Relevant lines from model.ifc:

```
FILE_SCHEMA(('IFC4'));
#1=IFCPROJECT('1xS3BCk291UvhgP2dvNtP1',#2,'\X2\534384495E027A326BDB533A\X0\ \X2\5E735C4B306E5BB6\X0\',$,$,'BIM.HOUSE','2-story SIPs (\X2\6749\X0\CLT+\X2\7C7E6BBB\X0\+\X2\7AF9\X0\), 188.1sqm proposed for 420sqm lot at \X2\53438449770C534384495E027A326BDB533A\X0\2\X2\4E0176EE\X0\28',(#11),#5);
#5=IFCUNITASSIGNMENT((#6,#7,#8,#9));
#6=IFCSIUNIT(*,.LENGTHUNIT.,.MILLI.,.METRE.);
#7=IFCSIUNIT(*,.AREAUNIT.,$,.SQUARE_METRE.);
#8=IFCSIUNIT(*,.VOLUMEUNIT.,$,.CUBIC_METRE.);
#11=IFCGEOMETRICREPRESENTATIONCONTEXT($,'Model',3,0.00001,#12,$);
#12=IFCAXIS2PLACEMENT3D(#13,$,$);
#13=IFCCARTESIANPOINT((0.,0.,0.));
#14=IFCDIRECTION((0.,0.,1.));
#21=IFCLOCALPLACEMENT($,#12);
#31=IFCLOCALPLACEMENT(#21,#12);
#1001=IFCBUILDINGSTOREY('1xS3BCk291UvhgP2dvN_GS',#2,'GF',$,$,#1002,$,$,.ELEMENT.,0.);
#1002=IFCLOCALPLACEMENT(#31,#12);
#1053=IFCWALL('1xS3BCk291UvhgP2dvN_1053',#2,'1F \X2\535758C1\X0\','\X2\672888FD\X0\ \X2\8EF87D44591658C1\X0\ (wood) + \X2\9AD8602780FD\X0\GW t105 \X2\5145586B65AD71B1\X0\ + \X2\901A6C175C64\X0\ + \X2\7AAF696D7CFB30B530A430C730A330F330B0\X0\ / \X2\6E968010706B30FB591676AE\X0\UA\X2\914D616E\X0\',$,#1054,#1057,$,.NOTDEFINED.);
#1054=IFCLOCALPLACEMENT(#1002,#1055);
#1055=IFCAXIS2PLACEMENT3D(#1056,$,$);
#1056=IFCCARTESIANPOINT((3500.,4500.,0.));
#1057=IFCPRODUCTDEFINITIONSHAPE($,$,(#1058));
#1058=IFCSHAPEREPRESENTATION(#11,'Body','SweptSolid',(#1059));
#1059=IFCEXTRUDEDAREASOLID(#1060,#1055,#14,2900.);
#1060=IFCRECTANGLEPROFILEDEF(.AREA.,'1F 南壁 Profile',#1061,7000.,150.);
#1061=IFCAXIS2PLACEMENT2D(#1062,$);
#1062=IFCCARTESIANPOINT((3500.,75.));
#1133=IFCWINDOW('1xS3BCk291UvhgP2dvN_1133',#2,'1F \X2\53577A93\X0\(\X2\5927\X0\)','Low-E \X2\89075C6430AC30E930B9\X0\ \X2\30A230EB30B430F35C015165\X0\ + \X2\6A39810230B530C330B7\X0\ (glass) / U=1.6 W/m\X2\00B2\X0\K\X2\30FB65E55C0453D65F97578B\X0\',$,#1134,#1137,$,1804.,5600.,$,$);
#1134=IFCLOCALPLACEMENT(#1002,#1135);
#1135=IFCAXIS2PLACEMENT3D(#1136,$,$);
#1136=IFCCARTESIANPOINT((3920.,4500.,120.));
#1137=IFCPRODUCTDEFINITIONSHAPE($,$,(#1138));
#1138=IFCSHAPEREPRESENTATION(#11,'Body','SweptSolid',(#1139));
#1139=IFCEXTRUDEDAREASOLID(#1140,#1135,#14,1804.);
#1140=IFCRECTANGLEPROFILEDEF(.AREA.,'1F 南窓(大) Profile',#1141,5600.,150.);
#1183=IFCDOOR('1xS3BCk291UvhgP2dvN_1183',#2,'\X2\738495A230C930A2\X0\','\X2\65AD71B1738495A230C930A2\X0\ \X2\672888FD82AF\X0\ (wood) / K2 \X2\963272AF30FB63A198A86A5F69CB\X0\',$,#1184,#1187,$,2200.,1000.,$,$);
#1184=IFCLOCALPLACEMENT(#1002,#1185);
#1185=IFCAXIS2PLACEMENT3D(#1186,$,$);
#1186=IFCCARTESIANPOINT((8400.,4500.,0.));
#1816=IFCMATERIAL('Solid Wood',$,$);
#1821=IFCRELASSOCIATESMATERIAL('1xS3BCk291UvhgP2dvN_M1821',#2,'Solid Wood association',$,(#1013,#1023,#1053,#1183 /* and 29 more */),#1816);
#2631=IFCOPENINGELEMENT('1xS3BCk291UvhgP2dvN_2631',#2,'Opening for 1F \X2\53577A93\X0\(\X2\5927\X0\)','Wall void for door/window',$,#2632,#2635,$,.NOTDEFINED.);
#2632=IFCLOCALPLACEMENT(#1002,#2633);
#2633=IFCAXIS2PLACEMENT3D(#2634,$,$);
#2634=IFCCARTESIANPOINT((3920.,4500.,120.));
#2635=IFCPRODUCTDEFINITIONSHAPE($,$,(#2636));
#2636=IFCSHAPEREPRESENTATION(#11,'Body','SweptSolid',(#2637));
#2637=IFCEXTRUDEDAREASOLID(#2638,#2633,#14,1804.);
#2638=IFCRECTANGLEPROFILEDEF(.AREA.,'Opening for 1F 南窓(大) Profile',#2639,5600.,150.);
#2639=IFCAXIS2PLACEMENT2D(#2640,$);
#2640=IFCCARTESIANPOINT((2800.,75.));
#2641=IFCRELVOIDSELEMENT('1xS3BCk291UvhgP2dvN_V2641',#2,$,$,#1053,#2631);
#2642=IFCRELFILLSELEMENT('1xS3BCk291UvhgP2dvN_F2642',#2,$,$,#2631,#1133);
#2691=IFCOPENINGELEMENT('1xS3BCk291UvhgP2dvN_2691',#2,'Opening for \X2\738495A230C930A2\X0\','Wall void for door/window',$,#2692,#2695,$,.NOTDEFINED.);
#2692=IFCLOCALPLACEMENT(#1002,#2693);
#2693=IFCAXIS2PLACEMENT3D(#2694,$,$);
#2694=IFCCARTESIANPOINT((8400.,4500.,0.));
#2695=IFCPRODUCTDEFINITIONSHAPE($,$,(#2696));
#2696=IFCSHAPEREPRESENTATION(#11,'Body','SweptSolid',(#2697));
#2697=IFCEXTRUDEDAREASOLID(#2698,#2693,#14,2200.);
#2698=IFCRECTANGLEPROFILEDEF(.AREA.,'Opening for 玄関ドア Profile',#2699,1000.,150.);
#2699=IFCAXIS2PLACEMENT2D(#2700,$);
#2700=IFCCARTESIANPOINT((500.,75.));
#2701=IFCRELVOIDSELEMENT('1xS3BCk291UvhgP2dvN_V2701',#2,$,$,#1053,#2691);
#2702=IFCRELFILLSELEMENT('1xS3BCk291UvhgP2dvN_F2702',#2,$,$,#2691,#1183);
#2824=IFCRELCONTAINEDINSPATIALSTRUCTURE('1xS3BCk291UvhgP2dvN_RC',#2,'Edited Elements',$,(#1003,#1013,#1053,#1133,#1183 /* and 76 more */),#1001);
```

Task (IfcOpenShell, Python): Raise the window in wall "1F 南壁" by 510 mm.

```python
import numpy as np
import ifcopenshell
import ifcopenshell.api.geometry
import ifcopenshell.util.placement
import ifcopenshell.util.unit

model = ifcopenshell.open("model.ifc")
unit_scale = ifcopenshell.util.unit.calculate_unit_scale(model)

window = model.by_guid("1xS3BCk291UvhgP2dvN_1133")
opening = window.FillsVoids[0].RelatingOpeningElement
dz = 510.0

shift = np.array([0.0, 0.0, dz])
# The window is not placed relative to its opening, so move both.
for product in (opening, window):
    matrix = ifcopenshell.util.placement.get_local_placement(product.ObjectPlacement)
    matrix[:3, 3] += shift
    ifcopenshell.api.geometry.edit_object_placement(model, product=product, matrix=matrix, is_si=False)

print(f"moved by {dz * unit_scale:+.3f} m")

model.write("model-out.ifc")
```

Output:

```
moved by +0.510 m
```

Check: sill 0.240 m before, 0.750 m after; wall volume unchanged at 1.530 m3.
